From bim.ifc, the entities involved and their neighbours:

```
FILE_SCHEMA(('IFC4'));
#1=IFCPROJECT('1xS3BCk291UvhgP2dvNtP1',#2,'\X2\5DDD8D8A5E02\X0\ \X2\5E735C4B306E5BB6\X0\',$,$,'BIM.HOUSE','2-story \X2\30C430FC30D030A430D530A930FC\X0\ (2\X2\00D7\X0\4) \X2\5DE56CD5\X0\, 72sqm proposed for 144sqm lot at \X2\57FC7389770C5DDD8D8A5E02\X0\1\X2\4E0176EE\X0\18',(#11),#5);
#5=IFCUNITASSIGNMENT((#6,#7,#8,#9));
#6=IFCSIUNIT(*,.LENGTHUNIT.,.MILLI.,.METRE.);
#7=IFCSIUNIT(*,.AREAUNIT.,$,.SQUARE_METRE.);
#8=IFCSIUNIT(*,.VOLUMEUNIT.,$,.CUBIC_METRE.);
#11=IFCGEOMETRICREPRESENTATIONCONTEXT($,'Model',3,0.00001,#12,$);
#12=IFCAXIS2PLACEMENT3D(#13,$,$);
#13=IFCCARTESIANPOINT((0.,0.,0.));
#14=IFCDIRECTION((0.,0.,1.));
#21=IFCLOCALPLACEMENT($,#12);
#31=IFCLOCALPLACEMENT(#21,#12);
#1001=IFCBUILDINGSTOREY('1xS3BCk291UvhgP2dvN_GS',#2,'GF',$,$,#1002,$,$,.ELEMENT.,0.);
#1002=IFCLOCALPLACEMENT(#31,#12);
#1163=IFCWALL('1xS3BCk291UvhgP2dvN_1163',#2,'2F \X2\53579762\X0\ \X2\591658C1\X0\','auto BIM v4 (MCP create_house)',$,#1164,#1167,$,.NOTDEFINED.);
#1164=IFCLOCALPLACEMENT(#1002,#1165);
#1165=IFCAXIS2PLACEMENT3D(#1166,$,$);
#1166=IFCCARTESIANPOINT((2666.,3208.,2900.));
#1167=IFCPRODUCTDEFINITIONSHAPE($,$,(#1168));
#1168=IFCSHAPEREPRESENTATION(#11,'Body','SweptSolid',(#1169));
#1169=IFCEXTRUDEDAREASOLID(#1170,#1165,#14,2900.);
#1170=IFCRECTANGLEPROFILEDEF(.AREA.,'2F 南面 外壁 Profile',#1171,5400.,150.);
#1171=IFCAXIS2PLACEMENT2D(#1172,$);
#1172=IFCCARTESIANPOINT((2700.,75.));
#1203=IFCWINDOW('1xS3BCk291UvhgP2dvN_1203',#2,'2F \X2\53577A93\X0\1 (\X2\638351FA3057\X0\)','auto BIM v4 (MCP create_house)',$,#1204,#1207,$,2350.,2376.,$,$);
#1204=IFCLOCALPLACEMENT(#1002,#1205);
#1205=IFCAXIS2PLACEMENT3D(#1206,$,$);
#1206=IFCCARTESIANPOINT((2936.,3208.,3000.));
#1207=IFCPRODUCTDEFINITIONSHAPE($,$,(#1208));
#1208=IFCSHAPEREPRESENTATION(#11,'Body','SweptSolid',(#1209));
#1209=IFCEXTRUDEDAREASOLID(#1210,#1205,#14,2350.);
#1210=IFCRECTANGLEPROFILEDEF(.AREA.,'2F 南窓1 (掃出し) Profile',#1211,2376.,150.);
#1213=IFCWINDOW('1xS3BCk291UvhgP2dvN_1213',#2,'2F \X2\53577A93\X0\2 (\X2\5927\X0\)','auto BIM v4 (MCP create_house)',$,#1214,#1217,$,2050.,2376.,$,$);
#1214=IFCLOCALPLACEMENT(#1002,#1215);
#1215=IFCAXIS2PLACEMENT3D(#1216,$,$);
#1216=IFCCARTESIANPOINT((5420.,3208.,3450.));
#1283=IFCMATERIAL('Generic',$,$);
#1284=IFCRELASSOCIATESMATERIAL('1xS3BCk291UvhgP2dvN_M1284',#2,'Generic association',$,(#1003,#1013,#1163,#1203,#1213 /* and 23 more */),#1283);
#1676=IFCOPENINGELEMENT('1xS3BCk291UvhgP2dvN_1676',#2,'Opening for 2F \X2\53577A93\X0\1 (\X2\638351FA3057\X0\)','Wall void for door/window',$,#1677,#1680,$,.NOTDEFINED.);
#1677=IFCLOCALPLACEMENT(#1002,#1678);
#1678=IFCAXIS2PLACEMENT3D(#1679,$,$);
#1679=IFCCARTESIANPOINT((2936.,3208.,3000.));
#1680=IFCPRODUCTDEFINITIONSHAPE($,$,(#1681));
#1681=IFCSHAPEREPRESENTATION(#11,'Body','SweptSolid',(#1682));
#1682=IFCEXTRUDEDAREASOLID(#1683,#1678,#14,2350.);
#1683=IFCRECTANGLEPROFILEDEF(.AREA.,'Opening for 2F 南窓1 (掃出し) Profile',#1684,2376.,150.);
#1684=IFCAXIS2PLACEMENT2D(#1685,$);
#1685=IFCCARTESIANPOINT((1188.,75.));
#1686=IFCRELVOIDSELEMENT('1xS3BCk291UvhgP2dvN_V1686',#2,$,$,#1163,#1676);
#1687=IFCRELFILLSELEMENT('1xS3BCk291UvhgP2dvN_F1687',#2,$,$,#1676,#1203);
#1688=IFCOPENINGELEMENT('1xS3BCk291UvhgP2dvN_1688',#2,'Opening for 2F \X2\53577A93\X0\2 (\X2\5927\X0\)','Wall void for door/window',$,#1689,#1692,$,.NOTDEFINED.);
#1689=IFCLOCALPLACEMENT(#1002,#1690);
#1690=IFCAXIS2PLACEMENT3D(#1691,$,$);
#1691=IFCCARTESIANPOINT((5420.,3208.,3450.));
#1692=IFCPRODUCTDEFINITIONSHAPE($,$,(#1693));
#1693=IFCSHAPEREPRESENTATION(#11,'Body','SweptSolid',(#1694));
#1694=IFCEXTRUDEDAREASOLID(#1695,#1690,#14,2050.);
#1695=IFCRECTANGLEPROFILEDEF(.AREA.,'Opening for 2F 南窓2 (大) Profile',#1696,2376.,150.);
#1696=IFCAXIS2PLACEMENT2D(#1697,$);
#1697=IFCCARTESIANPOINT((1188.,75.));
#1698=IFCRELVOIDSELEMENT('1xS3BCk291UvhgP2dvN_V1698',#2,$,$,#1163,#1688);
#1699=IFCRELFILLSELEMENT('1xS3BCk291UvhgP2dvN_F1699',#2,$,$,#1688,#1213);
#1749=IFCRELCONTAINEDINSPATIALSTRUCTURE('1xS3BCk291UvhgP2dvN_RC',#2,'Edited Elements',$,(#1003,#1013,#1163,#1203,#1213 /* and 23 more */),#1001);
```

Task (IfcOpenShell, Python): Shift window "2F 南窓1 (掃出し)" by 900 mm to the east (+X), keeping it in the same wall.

```python
import ifcopenshell
import ifcopenshell.api.geometry
import ifcopenshell.util.placement

model = ifcopenshell.open("bim.ifc")

window = model.by_guid("1xS3BCk291UvhgP2dvN_1203")
opening = window.FillsVoids[0].RelatingOpeningElement
wall = opening.VoidsElements[0].RelatingBuildingElement

wall_matrix = ifcopenshell.util.placement.get_local_placement(wall.ObjectPlacement)
shift = wall_matrix[:3, 0] * 900.0
before = ifcopenshell.util.placement.get_local_placement(window.ObjectPlacement)[:3, 3].copy()

# The window is not placed relative to its opening, so move both.
for product in (opening, window):
    matrix = ifcopenshell.util.placement.get_local_placement(product.ObjectPlacement)
    matrix[:3, 3] += shift
    ifcopenshell.api.geometry.edit_object_placement(model, product=product, matrix=matrix, is_si=False)

after = ifcopenshell.util.placement.get_local_placement(window.ObjectPlacement)[:3, 3]
print("window moved by", (after - before).round(3) + 0.0)

model.write("bim-out.ifc")
```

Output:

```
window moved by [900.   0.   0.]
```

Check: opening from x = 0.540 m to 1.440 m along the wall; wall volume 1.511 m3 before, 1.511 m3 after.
